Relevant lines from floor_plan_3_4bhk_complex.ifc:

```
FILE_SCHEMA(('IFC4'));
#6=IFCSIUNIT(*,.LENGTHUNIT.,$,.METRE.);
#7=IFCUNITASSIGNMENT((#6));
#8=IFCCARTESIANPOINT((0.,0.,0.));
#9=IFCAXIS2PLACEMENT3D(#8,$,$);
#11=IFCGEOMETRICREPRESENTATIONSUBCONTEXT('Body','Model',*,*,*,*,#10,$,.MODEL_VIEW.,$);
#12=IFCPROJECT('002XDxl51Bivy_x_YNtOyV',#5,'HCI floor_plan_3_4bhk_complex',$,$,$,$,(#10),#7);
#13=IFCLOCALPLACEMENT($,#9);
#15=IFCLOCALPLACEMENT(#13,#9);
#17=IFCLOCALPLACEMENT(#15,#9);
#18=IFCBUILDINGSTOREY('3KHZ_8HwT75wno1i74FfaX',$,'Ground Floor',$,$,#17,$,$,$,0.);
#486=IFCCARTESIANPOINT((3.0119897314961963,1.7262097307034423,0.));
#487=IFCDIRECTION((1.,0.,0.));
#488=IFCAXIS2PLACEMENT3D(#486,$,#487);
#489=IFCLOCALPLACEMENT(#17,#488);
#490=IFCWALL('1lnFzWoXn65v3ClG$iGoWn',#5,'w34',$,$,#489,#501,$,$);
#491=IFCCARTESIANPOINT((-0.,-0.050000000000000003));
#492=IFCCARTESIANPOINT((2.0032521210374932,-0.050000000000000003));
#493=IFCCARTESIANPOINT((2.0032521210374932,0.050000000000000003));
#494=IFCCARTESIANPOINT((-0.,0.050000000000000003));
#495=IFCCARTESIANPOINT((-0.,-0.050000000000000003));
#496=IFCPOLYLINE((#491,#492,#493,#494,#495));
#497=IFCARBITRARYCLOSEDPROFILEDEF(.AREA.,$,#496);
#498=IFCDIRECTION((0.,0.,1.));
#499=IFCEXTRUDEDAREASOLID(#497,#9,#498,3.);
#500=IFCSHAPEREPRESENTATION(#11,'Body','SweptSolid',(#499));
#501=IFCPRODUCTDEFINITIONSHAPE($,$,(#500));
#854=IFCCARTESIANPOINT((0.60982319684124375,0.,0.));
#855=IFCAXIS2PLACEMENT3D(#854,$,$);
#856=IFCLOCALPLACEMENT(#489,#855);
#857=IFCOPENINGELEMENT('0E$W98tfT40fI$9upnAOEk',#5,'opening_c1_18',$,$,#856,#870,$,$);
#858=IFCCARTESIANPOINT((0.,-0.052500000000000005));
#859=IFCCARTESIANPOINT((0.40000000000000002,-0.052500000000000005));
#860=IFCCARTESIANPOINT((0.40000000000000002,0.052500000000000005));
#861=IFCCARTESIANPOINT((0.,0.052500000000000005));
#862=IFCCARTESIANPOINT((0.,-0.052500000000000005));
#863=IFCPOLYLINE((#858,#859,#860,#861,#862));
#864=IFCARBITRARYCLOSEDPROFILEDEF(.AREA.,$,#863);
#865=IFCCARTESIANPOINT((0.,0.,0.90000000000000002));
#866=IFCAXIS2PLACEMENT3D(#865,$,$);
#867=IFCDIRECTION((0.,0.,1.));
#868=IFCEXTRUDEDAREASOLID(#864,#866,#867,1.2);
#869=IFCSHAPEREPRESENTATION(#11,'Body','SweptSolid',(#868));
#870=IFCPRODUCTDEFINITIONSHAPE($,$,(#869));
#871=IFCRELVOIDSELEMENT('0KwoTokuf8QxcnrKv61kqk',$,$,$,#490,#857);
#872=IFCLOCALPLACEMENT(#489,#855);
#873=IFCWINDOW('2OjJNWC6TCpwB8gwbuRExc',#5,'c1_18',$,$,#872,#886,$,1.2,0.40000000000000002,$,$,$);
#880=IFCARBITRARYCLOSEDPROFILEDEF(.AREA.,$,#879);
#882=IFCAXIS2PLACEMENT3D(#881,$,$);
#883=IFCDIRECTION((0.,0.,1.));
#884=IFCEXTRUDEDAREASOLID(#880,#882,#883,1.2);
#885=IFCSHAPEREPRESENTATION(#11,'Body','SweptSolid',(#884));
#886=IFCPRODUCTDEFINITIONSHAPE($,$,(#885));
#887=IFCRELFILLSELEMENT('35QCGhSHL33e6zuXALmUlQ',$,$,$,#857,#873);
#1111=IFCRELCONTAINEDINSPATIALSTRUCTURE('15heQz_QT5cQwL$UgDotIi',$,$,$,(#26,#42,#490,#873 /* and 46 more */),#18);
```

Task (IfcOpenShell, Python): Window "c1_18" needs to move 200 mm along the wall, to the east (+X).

```python
import ifcopenshell
import ifcopenshell.api.geometry
import ifcopenshell.util.placement
import ifcopenshell.util.unit

model = ifcopenshell.open("floor_plan_3_4bhk_complex.ifc")
unit_scale = ifcopenshell.util.unit.calculate_unit_scale(model)

window = model.by_guid("2OjJNWC6TCpwB8gwbuRExc")
opening = window.FillsVoids[0].RelatingOpeningElement
wall = opening.VoidsElements[0].RelatingBuildingElement

wall_matrix = ifcopenshell.util.placement.get_local_placement(wall.ObjectPlacement)
shift = wall_matrix[:3, 0] * 0.2 / unit_scale
before = ifcopenshell.util.placement.get_local_placement(window.ObjectPlacement)[:3, 3].copy()

# The window is not placed relative to its opening, so move both.
for product in (opening, window):
    matrix = ifcopenshell.util.placement.get_local_placement(product.ObjectPlacement)
    matrix[:3, 3] += shift
    ifcopenshell.api.geometry.edit_object_placement(model, product=product, matrix=matrix, is_si=False)

after = ifcopenshell.util.placement.get_local_placement(window.ObjectPlacement)[:3, 3]
print("window moved by", (after - before).round(3) + 0.0)

model.write("floor_plan_3_4bhk_complex-out.ifc")
```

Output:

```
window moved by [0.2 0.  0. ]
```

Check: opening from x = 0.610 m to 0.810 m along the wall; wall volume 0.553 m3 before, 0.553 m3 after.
